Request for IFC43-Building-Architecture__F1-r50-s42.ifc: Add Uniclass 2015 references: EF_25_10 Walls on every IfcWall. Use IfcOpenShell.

First a look at what the model holds.

```python
import ifcopenshell

model = ifcopenshell.open("IFC43-Building-Architecture__F1-r50-s42.ifc")
print(model.schema)
print("classifications:", [c.Name for c in model.by_type("IfcClassification")])
for ifc_class in ("IfcDoor", "IfcRoof", "IfcStair", "IfcWall", "IfcWindow"):
    print(ifc_class, len(model.by_type(ifc_class)))
```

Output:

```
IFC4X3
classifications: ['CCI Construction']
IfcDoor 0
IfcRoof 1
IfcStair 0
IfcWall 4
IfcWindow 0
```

```python
import ifcopenshell
import ifcopenshell.api.classification

model = ifcopenshell.open("IFC43-Building-Architecture__F1-r50-s42.ifc")

system = ifcopenshell.api.classification.add_classification(model, classification="Uniclass 2015")

codes = {
    "IfcWall": ("EF_25_10", "Walls"),
}
for ifc_class, (code, name) in codes.items():
    products = model.by_type(ifc_class)
    ifcopenshell.api.classification.add_reference(
        model, products=products, classification=system, identification=code, name=name
    )
    print(code, len(products))

model.write("IFC43-Building-Architecture__F1-r50-s42_updated.ifc")
```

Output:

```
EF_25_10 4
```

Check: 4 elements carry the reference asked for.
